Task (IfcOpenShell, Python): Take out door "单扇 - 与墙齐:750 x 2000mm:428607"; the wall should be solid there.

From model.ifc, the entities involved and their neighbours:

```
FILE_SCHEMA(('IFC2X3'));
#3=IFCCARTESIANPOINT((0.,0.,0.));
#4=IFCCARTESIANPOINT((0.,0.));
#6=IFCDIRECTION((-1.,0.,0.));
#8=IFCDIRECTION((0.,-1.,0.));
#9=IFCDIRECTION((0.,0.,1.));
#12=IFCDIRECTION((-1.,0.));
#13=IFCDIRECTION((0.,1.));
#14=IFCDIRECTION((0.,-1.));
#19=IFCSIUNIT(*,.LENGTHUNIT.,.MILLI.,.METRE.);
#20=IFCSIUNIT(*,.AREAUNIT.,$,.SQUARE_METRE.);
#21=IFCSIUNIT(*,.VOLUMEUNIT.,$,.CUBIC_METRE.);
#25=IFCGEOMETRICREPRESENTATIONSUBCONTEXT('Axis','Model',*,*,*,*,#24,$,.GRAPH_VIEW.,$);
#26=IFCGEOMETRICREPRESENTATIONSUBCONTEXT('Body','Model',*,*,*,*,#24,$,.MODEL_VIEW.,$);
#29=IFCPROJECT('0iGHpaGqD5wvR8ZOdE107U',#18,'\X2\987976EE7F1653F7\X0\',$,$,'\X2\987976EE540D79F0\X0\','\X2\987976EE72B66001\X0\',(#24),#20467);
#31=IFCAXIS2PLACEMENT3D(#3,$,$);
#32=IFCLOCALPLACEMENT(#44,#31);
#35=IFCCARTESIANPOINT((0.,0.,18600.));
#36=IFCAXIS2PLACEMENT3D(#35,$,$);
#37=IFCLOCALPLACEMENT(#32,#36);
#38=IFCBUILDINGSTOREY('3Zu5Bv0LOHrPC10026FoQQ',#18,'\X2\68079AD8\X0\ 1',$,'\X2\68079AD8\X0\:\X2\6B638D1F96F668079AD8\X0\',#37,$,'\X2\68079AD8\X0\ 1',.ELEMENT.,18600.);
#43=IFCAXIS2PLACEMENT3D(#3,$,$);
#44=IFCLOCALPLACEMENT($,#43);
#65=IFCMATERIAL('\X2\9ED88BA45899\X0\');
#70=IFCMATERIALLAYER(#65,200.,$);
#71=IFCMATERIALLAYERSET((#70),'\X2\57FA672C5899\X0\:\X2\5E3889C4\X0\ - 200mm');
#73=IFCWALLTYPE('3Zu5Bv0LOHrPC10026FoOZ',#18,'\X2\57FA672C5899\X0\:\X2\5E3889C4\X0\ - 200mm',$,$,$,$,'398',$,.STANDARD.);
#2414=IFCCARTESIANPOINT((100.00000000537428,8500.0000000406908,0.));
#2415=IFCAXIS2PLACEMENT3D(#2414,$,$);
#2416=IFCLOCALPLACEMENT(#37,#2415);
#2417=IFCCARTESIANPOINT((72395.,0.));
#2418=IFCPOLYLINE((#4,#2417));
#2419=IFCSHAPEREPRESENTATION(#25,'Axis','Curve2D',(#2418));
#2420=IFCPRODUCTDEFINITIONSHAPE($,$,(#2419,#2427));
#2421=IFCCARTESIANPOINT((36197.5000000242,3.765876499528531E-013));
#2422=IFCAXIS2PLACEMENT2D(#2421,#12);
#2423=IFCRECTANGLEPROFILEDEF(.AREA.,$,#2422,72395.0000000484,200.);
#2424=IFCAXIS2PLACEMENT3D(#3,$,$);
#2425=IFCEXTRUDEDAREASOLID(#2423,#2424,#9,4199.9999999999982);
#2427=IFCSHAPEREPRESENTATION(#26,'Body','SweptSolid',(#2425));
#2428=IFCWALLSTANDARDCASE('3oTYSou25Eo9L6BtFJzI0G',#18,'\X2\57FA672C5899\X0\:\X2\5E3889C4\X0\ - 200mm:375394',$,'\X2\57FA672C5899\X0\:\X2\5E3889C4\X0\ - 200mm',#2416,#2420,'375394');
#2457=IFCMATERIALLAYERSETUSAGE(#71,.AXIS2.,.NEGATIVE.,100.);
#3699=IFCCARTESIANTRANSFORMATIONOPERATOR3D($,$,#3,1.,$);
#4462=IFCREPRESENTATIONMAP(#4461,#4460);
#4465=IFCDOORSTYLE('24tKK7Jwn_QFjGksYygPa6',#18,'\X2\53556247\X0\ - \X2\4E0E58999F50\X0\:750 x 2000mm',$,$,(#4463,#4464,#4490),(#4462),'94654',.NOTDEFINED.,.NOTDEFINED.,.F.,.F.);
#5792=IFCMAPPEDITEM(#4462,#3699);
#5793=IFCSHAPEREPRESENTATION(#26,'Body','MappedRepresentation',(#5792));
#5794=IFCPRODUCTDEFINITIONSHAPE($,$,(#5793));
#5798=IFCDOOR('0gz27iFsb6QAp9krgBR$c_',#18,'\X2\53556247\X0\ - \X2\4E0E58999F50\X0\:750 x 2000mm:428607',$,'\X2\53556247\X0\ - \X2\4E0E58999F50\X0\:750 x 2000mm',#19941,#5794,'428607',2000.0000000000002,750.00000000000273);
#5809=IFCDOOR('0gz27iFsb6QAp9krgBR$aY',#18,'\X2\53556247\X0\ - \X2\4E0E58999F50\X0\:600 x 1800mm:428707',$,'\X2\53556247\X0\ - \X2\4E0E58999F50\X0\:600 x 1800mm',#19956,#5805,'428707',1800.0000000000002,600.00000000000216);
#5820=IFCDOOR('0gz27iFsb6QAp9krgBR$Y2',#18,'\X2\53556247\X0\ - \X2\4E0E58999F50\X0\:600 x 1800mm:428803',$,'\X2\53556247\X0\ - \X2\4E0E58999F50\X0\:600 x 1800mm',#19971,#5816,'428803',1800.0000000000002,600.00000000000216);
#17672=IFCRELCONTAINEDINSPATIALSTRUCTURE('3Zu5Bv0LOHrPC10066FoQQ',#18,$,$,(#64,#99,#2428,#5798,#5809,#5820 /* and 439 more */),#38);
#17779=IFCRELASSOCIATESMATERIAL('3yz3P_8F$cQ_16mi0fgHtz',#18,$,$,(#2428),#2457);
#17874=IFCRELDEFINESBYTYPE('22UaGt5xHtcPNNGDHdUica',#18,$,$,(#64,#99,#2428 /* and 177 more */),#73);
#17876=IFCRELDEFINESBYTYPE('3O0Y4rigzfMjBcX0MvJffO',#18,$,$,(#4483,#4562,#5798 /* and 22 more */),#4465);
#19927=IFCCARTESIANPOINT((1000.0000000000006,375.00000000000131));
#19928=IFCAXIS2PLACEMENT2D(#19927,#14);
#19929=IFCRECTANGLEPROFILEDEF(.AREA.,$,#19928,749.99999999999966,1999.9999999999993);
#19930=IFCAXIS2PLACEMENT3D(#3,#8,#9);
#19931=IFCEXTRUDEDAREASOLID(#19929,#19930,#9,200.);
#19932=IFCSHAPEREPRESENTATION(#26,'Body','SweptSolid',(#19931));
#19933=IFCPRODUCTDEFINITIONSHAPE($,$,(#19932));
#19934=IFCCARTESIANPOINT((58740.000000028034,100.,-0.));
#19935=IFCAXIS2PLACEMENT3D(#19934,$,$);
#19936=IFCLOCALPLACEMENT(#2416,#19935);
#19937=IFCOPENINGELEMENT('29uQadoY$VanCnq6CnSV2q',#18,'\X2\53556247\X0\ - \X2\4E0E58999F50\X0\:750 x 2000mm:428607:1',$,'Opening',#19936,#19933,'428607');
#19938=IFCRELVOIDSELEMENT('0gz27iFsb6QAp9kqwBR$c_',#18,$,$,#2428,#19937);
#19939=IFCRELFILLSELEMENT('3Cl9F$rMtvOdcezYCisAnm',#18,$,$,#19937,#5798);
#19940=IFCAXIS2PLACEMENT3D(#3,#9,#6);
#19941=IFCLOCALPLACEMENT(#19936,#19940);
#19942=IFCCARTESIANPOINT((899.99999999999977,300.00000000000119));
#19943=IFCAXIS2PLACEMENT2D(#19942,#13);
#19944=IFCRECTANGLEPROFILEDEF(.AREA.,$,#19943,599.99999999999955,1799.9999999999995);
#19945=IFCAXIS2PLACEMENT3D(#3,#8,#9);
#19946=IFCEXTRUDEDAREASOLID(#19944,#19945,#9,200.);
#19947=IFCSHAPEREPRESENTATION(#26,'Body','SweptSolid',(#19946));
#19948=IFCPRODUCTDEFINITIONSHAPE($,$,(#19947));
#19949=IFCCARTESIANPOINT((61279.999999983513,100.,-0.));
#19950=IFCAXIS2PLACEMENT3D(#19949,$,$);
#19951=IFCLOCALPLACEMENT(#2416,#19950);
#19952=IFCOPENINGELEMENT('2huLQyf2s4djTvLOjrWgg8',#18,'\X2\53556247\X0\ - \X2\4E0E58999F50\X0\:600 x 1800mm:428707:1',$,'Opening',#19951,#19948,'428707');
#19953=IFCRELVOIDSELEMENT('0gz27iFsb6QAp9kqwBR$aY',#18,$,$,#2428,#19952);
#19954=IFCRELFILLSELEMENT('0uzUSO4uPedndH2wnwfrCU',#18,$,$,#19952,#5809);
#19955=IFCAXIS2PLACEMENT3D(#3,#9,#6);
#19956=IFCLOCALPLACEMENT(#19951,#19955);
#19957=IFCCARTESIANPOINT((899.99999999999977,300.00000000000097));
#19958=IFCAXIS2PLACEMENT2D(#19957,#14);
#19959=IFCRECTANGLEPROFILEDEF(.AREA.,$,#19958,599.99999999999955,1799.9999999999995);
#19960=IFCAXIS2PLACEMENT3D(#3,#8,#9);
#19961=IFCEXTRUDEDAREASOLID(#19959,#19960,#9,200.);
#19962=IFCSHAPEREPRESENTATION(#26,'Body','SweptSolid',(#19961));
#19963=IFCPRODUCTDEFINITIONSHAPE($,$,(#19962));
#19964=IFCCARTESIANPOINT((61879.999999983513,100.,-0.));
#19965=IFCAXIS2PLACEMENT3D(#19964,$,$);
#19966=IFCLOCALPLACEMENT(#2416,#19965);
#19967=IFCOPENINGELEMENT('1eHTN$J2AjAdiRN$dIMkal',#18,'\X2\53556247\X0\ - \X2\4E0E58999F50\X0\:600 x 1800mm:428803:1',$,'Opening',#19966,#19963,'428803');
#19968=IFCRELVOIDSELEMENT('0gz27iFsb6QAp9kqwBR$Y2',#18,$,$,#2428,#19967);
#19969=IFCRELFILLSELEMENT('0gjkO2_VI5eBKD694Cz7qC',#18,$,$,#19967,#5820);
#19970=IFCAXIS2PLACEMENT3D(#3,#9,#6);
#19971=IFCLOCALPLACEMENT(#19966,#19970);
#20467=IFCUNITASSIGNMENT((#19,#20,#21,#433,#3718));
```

```python
import ifcopenshell
import ifcopenshell.api.feature
import ifcopenshell.api.root
import ifcopenshell.geom
import ifcopenshell.util.shape

model = ifcopenshell.open("model.ifc")
settings = ifcopenshell.geom.settings()


def volume(element):
    """Net volume in cubic metres, openings subtracted."""
    shape = ifcopenshell.geom.create_shape(settings, element)
    return ifcopenshell.util.shape.get_volume(shape.geometry)


door = model.by_guid("0gz27iFsb6QAp9krgBR$c_")
opening = door.FillsVoids[0].RelatingOpeningElement
wall = opening.VoidsElements[0].RelatingBuildingElement
before = volume(wall)

ifcopenshell.api.root.remove_product(model, product=door)
ifcopenshell.api.feature.remove_feature(model, feature=opening)

after = volume(wall)

print(f"wall volume {before:.3f} -> {after:.3f} m3")

model.write("model_edited.ifc")
```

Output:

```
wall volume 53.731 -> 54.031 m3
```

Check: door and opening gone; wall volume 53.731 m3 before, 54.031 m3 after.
